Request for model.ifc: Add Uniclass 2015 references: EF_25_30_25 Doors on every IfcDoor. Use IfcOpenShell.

First a look at what the model holds.

```python
import ifcopenshell

model = ifcopenshell.open("model.ifc")
print(model.schema)
print("classifications:", [c.Name for c in model.by_type("IfcClassification")])
for ifc_class in ("IfcDoor", "IfcRoof", "IfcStair", "IfcWall", "IfcWindow"):
    print(ifc_class, len(model.by_type(ifc_class)))
```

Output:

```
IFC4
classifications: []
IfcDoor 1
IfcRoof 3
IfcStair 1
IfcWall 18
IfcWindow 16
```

```python
import ifcopenshell
import ifcopenshell.api.classification

model = ifcopenshell.open("model.ifc")

system = ifcopenshell.api.classification.add_classification(model, classification="Uniclass 2015")

codes = {
    "IfcDoor": ("EF_25_30_25", "Doors"),
}
for ifc_class, (code, name) in codes.items():
    products = model.by_type(ifc_class)
    ifcopenshell.api.classification.add_reference(
        model, products=products, classification=system, identification=code, name=name
    )
    print(code, len(products))

model.write("model_rev.ifc")
```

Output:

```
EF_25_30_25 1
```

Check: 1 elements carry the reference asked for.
